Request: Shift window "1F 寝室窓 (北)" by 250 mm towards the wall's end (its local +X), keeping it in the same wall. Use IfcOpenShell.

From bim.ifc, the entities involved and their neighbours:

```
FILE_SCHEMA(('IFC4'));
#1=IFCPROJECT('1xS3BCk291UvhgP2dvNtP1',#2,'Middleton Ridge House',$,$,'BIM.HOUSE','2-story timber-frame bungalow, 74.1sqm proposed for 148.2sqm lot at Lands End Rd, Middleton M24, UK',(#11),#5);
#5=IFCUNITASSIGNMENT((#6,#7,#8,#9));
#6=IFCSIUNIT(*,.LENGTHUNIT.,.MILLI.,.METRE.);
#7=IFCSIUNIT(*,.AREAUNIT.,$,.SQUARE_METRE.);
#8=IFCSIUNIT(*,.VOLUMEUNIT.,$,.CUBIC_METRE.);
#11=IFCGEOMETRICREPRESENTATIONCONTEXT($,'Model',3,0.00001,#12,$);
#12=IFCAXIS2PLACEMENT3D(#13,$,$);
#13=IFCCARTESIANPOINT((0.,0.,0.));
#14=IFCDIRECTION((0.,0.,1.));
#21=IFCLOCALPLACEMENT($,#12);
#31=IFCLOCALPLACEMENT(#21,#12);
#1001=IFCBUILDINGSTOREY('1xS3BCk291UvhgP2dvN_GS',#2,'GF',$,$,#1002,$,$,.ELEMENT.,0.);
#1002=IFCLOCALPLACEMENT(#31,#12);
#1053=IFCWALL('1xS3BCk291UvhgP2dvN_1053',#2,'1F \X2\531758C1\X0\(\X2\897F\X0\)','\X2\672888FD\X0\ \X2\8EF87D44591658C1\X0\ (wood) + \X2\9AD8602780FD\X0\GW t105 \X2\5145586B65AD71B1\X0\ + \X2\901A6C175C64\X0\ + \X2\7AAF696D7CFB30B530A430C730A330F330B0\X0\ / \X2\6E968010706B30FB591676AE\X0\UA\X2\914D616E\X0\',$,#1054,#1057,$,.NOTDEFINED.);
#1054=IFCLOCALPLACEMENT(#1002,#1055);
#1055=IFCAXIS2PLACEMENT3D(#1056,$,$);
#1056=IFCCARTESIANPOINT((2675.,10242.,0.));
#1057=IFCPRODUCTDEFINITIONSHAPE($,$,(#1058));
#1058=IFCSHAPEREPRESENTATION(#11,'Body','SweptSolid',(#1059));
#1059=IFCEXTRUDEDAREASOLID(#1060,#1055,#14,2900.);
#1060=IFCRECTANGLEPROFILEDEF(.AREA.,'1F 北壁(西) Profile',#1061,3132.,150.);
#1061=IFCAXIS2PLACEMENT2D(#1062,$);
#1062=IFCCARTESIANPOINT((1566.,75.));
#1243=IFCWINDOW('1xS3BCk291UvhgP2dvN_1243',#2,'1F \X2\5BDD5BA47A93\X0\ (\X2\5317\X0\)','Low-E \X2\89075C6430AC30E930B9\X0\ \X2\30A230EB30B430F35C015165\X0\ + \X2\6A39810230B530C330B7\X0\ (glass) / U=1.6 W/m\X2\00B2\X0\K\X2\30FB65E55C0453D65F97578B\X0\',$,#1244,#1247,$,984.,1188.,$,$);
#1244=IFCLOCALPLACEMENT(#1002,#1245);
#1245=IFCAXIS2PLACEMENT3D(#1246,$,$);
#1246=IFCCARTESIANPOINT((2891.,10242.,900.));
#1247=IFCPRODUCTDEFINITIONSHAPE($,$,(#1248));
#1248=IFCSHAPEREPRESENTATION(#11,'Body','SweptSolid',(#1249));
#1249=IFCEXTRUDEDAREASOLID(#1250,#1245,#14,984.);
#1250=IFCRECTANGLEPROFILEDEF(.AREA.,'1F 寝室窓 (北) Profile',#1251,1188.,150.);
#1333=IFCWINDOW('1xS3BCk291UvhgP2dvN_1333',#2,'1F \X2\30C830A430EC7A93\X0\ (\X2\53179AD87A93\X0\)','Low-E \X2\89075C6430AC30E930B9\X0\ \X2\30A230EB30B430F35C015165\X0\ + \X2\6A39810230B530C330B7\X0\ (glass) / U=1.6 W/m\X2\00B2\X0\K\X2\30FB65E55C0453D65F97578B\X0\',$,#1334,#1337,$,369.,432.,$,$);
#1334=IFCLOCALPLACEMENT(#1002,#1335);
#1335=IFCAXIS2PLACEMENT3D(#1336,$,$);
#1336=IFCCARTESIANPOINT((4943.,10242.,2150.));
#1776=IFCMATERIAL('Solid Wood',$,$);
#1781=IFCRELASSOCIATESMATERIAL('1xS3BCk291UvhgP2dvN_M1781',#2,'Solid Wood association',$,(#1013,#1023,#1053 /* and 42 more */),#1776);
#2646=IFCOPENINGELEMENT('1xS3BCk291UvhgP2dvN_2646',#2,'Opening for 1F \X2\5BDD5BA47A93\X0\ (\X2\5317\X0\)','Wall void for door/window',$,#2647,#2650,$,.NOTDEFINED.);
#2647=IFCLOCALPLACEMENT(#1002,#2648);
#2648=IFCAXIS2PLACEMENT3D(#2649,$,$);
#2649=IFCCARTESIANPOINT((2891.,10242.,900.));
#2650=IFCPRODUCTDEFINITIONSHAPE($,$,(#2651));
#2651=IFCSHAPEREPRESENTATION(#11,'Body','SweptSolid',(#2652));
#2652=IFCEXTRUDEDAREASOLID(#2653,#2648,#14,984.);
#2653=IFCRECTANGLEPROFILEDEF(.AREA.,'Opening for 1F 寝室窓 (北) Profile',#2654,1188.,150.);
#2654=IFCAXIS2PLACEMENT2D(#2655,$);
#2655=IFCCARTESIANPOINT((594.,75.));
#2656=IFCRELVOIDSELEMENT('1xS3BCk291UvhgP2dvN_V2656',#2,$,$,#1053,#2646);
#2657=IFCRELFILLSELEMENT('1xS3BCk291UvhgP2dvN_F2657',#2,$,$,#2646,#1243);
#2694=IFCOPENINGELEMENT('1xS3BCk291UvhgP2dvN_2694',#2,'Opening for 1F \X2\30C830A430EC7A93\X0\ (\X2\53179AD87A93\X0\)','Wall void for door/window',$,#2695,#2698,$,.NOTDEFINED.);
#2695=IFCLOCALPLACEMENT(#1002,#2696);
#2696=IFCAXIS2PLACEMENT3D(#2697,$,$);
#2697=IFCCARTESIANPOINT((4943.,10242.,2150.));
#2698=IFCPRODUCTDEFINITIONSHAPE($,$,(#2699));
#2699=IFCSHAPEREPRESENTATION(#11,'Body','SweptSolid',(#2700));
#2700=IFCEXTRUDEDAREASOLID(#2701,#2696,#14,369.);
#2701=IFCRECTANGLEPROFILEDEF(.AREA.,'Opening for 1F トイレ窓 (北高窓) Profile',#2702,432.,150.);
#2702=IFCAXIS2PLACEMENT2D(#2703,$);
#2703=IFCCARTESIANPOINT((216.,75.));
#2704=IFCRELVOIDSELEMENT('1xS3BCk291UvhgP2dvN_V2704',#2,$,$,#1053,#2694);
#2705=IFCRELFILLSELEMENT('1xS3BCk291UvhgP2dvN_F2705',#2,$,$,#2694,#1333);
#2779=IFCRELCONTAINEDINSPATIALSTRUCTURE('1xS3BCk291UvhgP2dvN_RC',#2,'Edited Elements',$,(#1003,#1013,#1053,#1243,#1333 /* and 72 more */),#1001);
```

```python
import ifcopenshell
import ifcopenshell.api.geometry
import ifcopenshell.util.placement

model = ifcopenshell.open("bim.ifc")

window = model.by_guid("1xS3BCk291UvhgP2dvN_1243")
opening = window.FillsVoids[0].RelatingOpeningElement
wall = opening.VoidsElements[0].RelatingBuildingElement

wall_matrix = ifcopenshell.util.placement.get_local_placement(wall.ObjectPlacement)
shift = wall_matrix[:3, 0] * 250.0
before = ifcopenshell.util.placement.get_local_placement(window.ObjectPlacement)[:3, 3].copy()

# The window is not placed relative to its opening, so move both.
for product in (opening, window):
    matrix = ifcopenshell.util.placement.get_local_placement(product.ObjectPlacement)
    matrix[:3, 3] += shift
    ifcopenshell.api.geometry.edit_object_placement(model, product=product, matrix=matrix, is_si=False)

after = ifcopenshell.util.placement.get_local_placement(window.ObjectPlacement)[:3, 3]
print("window moved by", (after - before).round(3) + 0.0)

model.write("bim_updated.ifc")
```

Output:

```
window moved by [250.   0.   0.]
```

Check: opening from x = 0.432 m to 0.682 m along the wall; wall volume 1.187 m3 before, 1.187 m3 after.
